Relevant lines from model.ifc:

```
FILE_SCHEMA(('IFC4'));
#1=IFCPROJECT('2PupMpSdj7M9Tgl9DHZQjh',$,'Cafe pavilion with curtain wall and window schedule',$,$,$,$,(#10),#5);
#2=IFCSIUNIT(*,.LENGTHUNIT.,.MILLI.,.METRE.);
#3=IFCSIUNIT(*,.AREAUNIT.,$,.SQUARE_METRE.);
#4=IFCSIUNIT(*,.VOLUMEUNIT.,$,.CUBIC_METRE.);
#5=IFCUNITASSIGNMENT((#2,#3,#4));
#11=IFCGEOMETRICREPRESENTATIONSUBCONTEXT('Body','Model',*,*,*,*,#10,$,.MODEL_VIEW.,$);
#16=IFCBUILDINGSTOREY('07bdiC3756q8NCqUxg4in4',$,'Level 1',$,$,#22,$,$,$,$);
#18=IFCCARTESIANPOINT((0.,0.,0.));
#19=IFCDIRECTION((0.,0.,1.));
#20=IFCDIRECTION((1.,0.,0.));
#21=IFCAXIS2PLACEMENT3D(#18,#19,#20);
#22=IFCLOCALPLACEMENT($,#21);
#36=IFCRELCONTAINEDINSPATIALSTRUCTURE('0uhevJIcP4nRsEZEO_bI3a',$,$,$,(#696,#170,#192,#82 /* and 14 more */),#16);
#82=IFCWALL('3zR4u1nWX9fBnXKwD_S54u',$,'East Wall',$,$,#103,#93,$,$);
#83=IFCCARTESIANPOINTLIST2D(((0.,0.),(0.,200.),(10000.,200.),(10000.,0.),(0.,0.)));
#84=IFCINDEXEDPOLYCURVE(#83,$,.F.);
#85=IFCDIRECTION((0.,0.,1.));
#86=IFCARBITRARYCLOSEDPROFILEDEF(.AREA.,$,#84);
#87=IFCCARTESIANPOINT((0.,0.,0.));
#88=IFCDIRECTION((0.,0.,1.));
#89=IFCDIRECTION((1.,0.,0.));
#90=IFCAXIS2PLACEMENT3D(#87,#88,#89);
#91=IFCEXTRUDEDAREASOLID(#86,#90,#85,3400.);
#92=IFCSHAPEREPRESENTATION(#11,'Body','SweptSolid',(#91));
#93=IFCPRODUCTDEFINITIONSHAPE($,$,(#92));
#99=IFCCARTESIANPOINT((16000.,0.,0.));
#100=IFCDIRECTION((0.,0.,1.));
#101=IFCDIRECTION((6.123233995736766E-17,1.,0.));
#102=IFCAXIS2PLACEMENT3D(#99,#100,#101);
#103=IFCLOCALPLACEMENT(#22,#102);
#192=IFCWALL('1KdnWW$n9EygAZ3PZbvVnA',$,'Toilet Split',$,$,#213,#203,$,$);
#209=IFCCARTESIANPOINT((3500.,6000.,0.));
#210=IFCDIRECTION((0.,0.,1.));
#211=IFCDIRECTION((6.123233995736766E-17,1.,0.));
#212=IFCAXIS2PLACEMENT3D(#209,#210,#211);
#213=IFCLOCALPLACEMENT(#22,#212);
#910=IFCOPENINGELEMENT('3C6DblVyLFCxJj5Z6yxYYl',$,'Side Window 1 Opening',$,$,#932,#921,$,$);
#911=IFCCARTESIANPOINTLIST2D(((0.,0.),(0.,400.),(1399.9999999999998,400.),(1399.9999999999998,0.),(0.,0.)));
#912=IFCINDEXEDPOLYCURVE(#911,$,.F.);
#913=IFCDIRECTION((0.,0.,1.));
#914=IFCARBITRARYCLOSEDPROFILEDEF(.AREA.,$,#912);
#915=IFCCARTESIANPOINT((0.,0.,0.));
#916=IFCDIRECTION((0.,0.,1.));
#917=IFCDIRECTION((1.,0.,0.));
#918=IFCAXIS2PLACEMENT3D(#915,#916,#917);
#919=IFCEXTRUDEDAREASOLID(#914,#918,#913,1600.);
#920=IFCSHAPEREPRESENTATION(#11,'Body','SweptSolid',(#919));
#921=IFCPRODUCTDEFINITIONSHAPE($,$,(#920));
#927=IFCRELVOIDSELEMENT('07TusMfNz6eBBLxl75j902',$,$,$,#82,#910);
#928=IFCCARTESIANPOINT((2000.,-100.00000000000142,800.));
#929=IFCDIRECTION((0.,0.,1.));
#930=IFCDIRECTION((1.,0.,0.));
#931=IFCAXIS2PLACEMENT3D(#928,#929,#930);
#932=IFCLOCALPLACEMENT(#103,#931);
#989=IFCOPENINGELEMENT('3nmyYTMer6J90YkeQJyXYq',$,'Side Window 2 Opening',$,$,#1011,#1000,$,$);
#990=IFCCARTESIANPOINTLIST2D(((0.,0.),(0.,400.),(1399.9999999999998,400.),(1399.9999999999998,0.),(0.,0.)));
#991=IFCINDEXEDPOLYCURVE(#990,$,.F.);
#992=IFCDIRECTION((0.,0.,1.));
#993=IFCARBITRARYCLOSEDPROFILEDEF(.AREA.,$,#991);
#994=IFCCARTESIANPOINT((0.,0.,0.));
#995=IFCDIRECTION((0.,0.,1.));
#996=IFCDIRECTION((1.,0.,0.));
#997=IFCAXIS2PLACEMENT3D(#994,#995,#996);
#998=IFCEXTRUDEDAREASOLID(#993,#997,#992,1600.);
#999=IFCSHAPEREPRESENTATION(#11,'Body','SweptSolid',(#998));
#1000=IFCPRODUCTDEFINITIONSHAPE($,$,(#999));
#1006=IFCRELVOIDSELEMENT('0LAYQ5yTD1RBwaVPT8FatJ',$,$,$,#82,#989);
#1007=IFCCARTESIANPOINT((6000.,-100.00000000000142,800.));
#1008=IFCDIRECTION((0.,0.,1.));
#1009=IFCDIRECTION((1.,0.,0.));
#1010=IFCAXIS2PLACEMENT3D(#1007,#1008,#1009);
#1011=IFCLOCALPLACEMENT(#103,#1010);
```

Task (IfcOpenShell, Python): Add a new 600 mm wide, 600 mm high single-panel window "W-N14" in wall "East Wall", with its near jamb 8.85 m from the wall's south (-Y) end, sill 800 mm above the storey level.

```python
import numpy as np
import ifcopenshell
import ifcopenshell.api.feature
import ifcopenshell.api.geometry
import ifcopenshell.api.root
import ifcopenshell.api.spatial
import ifcopenshell.geom
import ifcopenshell.util.element
import ifcopenshell.util.placement
import ifcopenshell.util.representation
import ifcopenshell.util.shape
import ifcopenshell.util.unit

model = ifcopenshell.open("model.ifc")
unit_scale = ifcopenshell.util.unit.calculate_unit_scale(model)
settings = ifcopenshell.geom.settings()


def volume(element):
    """Net volume in cubic metres, openings subtracted."""
    shape = ifcopenshell.geom.create_shape(settings, element)
    return ifcopenshell.util.shape.get_volume(shape.geometry)


wall = model.by_id(82)
storey = ifcopenshell.util.element.get_container(wall, ifc_class="IfcBuildingStorey")
context = ifcopenshell.util.representation.get_context(model, "Model", "Body", "MODEL_VIEW")
before = volume(wall)

width, height, from_end, sill = 0.6, 0.6, 8.85, 0.8  # metres

# The wall runs along its own X axis, and the end named is its -X end.
wall_shape = ifcopenshell.geom.create_shape(settings, wall)
x, y, z = ifcopenshell.util.shape.get_vertices(wall_shape.geometry).T
start = x.min() + from_end
face, thickness = float(y.min()), float(y.max() - y.min())
wall_matrix = ifcopenshell.util.placement.get_local_placement(wall.ObjectPlacement)
level = ifcopenshell.util.placement.get_local_placement(storey.ObjectPlacement)[2, 3]


def in_wall(x, y):
    """Placement at x, y metres in the wall's axes, at sill height."""
    matrix = wall_matrix.copy()
    matrix[:, 3] = wall_matrix @ np.array([x / unit_scale, y / unit_scale, 0.0, 1.0])
    matrix[2, 3] = level + sill / unit_scale
    return matrix


# Opening: a box that overshoots both wall faces by 50 mm.
opening = ifcopenshell.api.root.create_entity(model, ifc_class="IfcOpeningElement", predefined_type="OPENING")
box = ifcopenshell.api.geometry.add_wall_representation(
    model, context=context, length=width, height=height, thickness=thickness + 0.1
)
ifcopenshell.api.geometry.assign_representation(model, product=opening, representation=box)
ifcopenshell.api.geometry.edit_object_placement(model, product=opening, matrix=in_wall(start, face - 0.05), is_si=False)
ifcopenshell.api.feature.add_feature(model, feature=opening, element=wall)

window = ifcopenshell.api.root.create_entity(model, ifc_class="IfcWindow", name="W-N14", predefined_type="WINDOW")
window.OverallWidth, window.OverallHeight = width / unit_scale, height / unit_scale
window.PartitioningType = "SINGLE_PANEL"
body = ifcopenshell.api.geometry.add_window_representation(
    model,
    context=context,
    overall_width=window.OverallWidth,
    overall_height=window.OverallHeight,
    partition_type="SINGLE_PANEL",
)
ifcopenshell.api.geometry.assign_representation(model, product=window, representation=body)
ifcopenshell.api.spatial.assign_container(model, products=[window], relating_structure=storey)
ifcopenshell.api.feature.add_filling(model, opening=opening, element=window)

# Centre the window in the wall's thickness.
ifcopenshell.api.geometry.edit_object_placement(model, product=window, matrix=in_wall(start, face), is_si=False)
window_shape = ifcopenshell.geom.create_shape(settings, window)
depth = ifcopenshell.util.shape.get_vertices(window_shape.geometry)[:, 1]
offset = face + thickness / 2 - (depth.min() + depth.max()) / 2
ifcopenshell.api.geometry.edit_object_placement(model, product=window, matrix=in_wall(start, offset), is_si=False)

after = volume(wall)

print(f"wall volume {before:.3f} -> {after:.3f} m3")

model.write("model_updated.ifc")
```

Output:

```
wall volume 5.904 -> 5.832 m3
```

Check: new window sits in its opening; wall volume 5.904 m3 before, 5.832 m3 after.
